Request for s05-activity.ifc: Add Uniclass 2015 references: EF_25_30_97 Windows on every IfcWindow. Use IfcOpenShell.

First a look at what the model holds.

```python
import ifcopenshell

model = ifcopenshell.open("s05-activity.ifc")
print(model.schema)
print("classifications:", [c.Name for c in model.by_type("IfcClassification")])
for ifc_class in ("IfcDoor", "IfcRoof", "IfcStair", "IfcWall", "IfcWindow"):
    print(ifc_class, len(model.by_type(ifc_class)))
```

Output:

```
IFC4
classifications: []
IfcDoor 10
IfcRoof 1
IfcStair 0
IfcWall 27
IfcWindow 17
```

```python
import ifcopenshell
import ifcopenshell.api.classification

model = ifcopenshell.open("s05-activity.ifc")

system = ifcopenshell.api.classification.add_classification(model, classification="Uniclass 2015")

codes = {
    "IfcWindow": ("EF_25_30_97", "Windows"),
}
for ifc_class, (code, name) in codes.items():
    products = model.by_type(ifc_class)
    ifcopenshell.api.classification.add_reference(
        model, products=products, classification=system, identification=code, name=name
    )
    print(code, len(products))

model.write("s05-activity_v2.ifc")
```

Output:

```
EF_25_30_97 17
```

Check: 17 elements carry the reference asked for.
